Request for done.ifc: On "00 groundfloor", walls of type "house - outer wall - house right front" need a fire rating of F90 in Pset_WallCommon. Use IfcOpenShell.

First a look at what the model holds.

```python
import ifcopenshell
import ifcopenshell.util.element

model = ifcopenshell.open("done.ifc")
print(model.schema)
storey = next(s for s in model.by_type("IfcBuildingStorey") if s.Name == "00 groundfloor")
walls = [e for e in ifcopenshell.util.element.get_decomposition(storey) if e.is_a("IfcWall")]
seen = {}
for e in walls:
    element_type = ifcopenshell.util.element.get_type(e)
    key = (element_type.Name if element_type != e and element_type else None, ifcopenshell.util.element.get_pset(e, "Pset_WallCommon", "FireRating"))
    seen[key] = seen.get(key, 0) + 1
for (name, value), count in sorted(seen.items(), key=str):
    print(count, "x", name, "|", value)
```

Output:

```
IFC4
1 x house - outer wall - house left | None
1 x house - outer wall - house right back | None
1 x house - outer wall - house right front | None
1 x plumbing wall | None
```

```python
import ifcopenshell
import ifcopenshell.api.pset
import ifcopenshell.util.element

model = ifcopenshell.open("done.ifc")

storey = next(s for s in model.by_type("IfcBuildingStorey") if s.Name == "00 groundfloor")
walls = [e for e in ifcopenshell.util.element.get_decomposition(storey) if e.is_a("IfcWall")]

count = 0
for e in walls:
    element_type = ifcopenshell.util.element.get_type(e)
    if element_type in (None, e) or element_type.Name != "house - outer wall - house right front":
        continue
    # add_pset returns the element's existing set when there is one.
    pset = ifcopenshell.api.pset.add_pset(model, product=e, name="Pset_WallCommon")
    ifcopenshell.api.pset.edit_pset(model, pset=pset, properties={"FireRating": "F90"})
    count += 1

print(count, "walls updated")

model.write("done_edited.ifc")
```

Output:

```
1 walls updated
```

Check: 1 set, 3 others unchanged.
